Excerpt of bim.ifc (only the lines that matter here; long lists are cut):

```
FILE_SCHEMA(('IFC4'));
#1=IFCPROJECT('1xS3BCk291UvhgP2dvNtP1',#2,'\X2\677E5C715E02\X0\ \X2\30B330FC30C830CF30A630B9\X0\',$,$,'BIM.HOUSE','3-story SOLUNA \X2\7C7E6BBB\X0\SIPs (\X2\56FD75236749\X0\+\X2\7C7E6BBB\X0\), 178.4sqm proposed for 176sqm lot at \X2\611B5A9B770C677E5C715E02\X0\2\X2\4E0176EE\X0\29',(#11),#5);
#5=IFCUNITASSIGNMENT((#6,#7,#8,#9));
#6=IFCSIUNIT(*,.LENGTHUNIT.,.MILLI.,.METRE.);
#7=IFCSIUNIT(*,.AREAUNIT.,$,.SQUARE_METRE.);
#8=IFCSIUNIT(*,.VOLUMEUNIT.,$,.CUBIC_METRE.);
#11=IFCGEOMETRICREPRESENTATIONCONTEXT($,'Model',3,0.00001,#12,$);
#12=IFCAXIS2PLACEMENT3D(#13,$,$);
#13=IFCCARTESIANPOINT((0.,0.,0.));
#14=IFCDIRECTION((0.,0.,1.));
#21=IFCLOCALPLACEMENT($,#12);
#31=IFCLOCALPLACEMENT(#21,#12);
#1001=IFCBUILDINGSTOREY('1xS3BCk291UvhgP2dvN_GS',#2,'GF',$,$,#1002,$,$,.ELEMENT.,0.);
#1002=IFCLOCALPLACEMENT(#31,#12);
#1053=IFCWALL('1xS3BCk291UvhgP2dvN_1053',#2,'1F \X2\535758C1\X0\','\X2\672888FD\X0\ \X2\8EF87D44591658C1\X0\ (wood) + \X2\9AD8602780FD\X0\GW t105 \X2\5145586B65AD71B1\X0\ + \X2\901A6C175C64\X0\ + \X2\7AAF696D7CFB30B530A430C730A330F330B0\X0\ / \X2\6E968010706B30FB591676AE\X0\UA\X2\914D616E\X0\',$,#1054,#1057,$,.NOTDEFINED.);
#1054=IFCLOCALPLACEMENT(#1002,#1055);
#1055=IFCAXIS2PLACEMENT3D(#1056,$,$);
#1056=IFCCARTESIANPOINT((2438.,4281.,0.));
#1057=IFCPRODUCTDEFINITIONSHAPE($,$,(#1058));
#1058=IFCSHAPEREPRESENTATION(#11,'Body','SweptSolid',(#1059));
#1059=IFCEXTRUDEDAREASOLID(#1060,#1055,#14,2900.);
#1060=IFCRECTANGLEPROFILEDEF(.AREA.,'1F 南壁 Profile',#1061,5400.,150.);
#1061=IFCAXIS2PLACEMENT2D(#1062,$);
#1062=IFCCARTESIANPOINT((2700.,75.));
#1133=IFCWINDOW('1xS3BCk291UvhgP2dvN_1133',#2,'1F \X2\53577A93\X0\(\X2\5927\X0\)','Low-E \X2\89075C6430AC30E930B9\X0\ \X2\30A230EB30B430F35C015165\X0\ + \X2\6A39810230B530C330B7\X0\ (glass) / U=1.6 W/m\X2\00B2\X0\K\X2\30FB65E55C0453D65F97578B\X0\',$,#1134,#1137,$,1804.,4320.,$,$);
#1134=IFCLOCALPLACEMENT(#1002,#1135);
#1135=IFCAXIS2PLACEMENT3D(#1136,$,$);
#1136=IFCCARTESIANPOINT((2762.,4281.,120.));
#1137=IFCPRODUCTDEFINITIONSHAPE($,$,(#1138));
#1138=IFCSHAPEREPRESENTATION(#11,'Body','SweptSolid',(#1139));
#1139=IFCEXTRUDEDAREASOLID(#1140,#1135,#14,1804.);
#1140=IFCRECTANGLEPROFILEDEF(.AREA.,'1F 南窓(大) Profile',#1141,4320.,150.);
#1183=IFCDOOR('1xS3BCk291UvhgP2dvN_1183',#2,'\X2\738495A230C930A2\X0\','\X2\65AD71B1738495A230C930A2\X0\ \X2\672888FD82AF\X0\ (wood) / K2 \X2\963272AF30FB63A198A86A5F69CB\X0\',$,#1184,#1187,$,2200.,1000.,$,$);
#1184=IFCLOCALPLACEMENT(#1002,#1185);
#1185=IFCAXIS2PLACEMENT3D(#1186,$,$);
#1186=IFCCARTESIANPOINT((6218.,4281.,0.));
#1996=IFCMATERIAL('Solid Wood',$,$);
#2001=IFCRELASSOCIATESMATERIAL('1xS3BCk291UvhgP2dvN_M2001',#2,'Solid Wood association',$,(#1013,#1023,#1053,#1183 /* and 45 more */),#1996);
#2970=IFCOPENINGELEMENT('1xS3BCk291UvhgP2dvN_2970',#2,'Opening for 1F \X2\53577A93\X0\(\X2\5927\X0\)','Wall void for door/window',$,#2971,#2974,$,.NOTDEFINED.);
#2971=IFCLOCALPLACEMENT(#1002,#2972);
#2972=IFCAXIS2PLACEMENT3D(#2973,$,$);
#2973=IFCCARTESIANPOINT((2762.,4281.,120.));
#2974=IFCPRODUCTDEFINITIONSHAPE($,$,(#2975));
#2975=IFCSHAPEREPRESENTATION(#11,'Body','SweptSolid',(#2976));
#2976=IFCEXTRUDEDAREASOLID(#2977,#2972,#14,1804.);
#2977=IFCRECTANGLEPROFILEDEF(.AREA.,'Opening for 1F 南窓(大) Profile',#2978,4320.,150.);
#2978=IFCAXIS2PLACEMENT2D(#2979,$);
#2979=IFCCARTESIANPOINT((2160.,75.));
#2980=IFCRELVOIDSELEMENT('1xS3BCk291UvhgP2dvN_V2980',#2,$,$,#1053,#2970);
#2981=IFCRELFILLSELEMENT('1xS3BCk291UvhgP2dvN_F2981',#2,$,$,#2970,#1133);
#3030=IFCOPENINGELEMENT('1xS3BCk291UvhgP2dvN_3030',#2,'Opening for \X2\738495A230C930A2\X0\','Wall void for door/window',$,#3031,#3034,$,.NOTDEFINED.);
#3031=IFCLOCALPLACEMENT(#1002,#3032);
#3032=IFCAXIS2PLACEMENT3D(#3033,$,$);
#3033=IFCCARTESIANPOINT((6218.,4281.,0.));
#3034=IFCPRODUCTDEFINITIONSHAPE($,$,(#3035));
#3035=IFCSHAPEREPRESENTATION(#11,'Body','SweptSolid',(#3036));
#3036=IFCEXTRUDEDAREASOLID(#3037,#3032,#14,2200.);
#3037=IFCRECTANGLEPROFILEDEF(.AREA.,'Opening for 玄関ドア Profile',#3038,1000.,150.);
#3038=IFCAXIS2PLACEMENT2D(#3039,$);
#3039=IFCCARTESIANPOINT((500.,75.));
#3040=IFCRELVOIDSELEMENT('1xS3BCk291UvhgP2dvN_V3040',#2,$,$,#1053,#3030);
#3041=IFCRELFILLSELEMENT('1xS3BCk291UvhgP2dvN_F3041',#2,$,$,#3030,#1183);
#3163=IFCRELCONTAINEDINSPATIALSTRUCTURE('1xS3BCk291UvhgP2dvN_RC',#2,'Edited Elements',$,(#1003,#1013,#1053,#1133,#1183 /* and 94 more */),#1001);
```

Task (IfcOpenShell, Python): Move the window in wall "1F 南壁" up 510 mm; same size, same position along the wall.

```python
import numpy as np
import ifcopenshell
import ifcopenshell.api.geometry
import ifcopenshell.util.placement
import ifcopenshell.util.unit

model = ifcopenshell.open("bim.ifc")
unit_scale = ifcopenshell.util.unit.calculate_unit_scale(model)

window = model.by_guid("1xS3BCk291UvhgP2dvN_1133")
opening = window.FillsVoids[0].RelatingOpeningElement
dz = 510.0

shift = np.array([0.0, 0.0, dz])
# The window is not placed relative to its opening, so move both.
for product in (opening, window):
    matrix = ifcopenshell.util.placement.get_local_placement(product.ObjectPlacement)
    matrix[:3, 3] += shift
    ifcopenshell.api.geometry.edit_object_placement(model, product=product, matrix=matrix, is_si=False)

print(f"moved by {dz * unit_scale:+.3f} m")

model.write("bim_edited.ifc")
```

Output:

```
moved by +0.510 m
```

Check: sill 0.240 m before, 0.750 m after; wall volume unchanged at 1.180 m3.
